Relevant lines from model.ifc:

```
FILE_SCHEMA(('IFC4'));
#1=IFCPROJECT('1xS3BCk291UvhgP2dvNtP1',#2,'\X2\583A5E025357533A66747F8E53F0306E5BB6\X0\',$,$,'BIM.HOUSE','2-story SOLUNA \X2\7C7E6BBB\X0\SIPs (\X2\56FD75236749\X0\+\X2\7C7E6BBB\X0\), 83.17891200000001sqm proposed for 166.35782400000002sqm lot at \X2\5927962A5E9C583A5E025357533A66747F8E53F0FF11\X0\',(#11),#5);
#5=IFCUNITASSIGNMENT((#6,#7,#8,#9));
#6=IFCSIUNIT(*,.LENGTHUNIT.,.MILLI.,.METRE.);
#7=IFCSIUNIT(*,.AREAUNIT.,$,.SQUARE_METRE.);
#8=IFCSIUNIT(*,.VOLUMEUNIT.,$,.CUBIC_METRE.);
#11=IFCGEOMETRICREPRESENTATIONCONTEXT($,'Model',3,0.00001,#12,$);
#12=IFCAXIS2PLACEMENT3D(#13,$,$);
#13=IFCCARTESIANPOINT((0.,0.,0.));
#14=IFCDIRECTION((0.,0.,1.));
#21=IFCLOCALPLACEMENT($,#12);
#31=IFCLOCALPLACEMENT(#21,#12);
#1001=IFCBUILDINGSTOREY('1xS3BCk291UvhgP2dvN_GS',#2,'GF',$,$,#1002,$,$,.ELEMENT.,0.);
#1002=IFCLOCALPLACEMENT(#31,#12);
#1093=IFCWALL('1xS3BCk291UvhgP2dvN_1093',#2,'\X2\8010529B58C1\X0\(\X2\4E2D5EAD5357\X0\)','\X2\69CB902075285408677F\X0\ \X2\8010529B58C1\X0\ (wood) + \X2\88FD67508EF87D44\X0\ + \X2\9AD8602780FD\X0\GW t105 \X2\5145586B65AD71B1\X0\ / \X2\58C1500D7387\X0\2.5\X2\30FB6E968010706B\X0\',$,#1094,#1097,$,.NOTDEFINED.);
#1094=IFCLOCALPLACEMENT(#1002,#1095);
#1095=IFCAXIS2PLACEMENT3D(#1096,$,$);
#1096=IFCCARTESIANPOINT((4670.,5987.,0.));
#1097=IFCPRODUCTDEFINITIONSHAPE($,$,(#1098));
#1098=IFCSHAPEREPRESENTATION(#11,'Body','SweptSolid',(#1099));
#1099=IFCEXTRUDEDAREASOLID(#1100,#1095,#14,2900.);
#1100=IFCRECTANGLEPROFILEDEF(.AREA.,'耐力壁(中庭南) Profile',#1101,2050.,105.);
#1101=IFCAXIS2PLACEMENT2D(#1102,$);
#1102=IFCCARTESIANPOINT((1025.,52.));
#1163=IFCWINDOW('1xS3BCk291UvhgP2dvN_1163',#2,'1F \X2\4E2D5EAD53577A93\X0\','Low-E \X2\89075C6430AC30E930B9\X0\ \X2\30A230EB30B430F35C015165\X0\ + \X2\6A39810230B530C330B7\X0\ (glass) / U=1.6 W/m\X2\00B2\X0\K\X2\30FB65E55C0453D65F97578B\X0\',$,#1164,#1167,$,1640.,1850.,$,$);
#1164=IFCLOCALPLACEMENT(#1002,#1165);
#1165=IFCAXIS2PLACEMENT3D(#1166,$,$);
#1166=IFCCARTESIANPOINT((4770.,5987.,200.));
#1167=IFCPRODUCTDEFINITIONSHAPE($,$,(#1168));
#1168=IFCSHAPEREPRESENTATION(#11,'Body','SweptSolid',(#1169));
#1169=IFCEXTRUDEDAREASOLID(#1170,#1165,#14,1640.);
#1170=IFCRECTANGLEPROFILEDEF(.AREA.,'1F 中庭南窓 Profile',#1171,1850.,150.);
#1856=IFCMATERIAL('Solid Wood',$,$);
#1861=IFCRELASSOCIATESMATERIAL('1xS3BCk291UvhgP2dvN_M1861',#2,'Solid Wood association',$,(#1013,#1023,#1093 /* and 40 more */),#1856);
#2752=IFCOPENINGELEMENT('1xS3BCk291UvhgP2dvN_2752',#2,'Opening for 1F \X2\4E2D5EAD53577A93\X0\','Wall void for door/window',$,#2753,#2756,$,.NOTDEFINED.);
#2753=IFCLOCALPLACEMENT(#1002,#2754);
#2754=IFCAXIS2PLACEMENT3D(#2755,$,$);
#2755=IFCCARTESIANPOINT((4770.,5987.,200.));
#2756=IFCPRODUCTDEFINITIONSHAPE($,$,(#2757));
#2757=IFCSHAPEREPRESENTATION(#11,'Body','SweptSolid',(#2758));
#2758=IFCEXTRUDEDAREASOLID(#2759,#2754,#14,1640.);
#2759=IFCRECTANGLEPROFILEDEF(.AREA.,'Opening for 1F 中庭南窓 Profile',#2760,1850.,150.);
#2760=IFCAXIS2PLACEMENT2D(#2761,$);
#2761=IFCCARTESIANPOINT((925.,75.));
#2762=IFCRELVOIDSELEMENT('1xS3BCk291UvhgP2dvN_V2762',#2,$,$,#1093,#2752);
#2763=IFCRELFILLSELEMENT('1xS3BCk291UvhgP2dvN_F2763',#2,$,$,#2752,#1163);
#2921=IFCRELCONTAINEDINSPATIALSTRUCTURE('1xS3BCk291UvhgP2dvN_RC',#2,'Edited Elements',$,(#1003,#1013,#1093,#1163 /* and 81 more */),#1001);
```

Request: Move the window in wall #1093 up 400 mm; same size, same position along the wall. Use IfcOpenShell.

```python
import numpy as np
import ifcopenshell
import ifcopenshell.api.geometry
import ifcopenshell.util.placement
import ifcopenshell.util.unit

model = ifcopenshell.open("model.ifc")
unit_scale = ifcopenshell.util.unit.calculate_unit_scale(model)

window = model.by_guid("1xS3BCk291UvhgP2dvN_1163")
opening = window.FillsVoids[0].RelatingOpeningElement
dz = 0.4 / unit_scale

shift = np.array([0.0, 0.0, dz])
# The window is not placed relative to its opening, so move both.
for product in (opening, window):
    matrix = ifcopenshell.util.placement.get_local_placement(product.ObjectPlacement)
    matrix[:3, 3] += shift
    ifcopenshell.api.geometry.edit_object_placement(model, product=product, matrix=matrix, is_si=False)

print(f"moved by {dz * unit_scale:+.3f} m")

model.write("model_rev.ifc")
```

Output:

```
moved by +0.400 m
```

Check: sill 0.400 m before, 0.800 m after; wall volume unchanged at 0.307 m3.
